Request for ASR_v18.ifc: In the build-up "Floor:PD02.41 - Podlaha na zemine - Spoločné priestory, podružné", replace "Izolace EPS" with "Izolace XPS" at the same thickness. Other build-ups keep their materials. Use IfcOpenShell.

First a look at what the model holds.

```python
import ifcopenshell
import ifcopenshell.util.element

model = ifcopenshell.open("ASR_v18.ifc")
print(model.schema)
for layer_set in model.by_type("IfcMaterialLayerSet"):
    if layer_set.LayerSetName == "Floor:PD02.41 - Podlaha na zemine - Spoločné priestory, podružné":
        for layer in layer_set.MaterialLayers:
            print(layer.id(), layer.Material and layer.Material.Name, layer.LayerThickness, sep=" | ")
        print(len(ifcopenshell.util.element.get_elements_by_material(model, layer_set)), "elements and types use it")
print(sorted(m.Name for m in model.by_type("IfcMaterial") if m.Name)[:60])
```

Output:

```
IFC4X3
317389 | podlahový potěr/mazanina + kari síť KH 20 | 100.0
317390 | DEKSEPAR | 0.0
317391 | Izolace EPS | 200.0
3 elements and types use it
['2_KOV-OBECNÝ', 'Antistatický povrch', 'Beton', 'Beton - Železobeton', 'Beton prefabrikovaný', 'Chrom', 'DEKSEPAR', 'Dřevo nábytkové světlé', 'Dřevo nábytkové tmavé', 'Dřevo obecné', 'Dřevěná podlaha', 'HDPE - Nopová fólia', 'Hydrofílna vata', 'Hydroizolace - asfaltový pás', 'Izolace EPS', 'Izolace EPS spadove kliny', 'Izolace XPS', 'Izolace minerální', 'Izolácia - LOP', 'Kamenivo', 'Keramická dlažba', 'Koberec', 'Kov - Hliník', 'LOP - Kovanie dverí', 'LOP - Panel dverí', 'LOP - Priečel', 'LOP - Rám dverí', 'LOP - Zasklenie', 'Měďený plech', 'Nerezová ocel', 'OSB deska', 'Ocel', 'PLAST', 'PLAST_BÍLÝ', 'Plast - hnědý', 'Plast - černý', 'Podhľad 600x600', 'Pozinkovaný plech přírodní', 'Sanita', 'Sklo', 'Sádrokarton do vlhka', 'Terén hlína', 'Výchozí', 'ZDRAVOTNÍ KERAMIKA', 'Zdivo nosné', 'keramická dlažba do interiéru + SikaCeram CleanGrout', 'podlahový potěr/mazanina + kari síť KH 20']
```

```python
import ifcopenshell
import ifcopenshell.api.material

model = ifcopenshell.open("ASR_v18.ifc")

layer_set = next(s for s in model.by_type("IfcMaterialLayerSet") if s.LayerSetName == "Floor:PD02.41 - Podlaha na zemine - Spoločné priestory, podružné")
layer = next(l for l in layer_set.MaterialLayers if l.Material and l.Material.Name == "Izolace EPS")
material = next(m for m in model.by_type("IfcMaterial") if m.Name == "Izolace XPS")

# Point this one layer at the other material; renaming the old one would change it everywhere.
ifcopenshell.api.material.edit_layer(model, layer=layer, attributes={"Name": material.Name}, material=material)

print([l.Material.Name if l.Material else None for l in layer_set.MaterialLayers])

model.write("ASR_v18_rev.ifc")
```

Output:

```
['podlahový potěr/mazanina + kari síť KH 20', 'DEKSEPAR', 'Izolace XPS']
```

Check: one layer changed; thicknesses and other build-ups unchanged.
